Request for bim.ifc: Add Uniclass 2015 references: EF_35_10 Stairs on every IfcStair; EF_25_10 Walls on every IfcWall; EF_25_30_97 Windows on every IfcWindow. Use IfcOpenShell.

First a look at what the model holds.

```python
import ifcopenshell

model = ifcopenshell.open("bim.ifc")
print(model.schema)
print("classifications:", [c.Name for c in model.by_type("IfcClassification")])
for ifc_class in ("IfcDoor", "IfcRoof", "IfcStair", "IfcWall", "IfcWindow"):
    print(ifc_class, len(model.by_type(ifc_class)))
```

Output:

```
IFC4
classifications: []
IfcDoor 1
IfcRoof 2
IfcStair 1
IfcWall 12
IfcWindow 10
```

```python
import ifcopenshell
import ifcopenshell.api.classification

model = ifcopenshell.open("bim.ifc")

system = ifcopenshell.api.classification.add_classification(model, classification="Uniclass 2015")

codes = {
    "IfcStair": ("EF_35_10", "Stairs"),
    "IfcWall": ("EF_25_10", "Walls"),
    "IfcWindow": ("EF_25_30_97", "Windows"),
}
for ifc_class, (code, name) in codes.items():
    products = model.by_type(ifc_class)
    ifcopenshell.api.classification.add_reference(
        model, products=products, classification=system, identification=code, name=name
    )
    print(code, len(products))

model.write("bim_edited.ifc")
```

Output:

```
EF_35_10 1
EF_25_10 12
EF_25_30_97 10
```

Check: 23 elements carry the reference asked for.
